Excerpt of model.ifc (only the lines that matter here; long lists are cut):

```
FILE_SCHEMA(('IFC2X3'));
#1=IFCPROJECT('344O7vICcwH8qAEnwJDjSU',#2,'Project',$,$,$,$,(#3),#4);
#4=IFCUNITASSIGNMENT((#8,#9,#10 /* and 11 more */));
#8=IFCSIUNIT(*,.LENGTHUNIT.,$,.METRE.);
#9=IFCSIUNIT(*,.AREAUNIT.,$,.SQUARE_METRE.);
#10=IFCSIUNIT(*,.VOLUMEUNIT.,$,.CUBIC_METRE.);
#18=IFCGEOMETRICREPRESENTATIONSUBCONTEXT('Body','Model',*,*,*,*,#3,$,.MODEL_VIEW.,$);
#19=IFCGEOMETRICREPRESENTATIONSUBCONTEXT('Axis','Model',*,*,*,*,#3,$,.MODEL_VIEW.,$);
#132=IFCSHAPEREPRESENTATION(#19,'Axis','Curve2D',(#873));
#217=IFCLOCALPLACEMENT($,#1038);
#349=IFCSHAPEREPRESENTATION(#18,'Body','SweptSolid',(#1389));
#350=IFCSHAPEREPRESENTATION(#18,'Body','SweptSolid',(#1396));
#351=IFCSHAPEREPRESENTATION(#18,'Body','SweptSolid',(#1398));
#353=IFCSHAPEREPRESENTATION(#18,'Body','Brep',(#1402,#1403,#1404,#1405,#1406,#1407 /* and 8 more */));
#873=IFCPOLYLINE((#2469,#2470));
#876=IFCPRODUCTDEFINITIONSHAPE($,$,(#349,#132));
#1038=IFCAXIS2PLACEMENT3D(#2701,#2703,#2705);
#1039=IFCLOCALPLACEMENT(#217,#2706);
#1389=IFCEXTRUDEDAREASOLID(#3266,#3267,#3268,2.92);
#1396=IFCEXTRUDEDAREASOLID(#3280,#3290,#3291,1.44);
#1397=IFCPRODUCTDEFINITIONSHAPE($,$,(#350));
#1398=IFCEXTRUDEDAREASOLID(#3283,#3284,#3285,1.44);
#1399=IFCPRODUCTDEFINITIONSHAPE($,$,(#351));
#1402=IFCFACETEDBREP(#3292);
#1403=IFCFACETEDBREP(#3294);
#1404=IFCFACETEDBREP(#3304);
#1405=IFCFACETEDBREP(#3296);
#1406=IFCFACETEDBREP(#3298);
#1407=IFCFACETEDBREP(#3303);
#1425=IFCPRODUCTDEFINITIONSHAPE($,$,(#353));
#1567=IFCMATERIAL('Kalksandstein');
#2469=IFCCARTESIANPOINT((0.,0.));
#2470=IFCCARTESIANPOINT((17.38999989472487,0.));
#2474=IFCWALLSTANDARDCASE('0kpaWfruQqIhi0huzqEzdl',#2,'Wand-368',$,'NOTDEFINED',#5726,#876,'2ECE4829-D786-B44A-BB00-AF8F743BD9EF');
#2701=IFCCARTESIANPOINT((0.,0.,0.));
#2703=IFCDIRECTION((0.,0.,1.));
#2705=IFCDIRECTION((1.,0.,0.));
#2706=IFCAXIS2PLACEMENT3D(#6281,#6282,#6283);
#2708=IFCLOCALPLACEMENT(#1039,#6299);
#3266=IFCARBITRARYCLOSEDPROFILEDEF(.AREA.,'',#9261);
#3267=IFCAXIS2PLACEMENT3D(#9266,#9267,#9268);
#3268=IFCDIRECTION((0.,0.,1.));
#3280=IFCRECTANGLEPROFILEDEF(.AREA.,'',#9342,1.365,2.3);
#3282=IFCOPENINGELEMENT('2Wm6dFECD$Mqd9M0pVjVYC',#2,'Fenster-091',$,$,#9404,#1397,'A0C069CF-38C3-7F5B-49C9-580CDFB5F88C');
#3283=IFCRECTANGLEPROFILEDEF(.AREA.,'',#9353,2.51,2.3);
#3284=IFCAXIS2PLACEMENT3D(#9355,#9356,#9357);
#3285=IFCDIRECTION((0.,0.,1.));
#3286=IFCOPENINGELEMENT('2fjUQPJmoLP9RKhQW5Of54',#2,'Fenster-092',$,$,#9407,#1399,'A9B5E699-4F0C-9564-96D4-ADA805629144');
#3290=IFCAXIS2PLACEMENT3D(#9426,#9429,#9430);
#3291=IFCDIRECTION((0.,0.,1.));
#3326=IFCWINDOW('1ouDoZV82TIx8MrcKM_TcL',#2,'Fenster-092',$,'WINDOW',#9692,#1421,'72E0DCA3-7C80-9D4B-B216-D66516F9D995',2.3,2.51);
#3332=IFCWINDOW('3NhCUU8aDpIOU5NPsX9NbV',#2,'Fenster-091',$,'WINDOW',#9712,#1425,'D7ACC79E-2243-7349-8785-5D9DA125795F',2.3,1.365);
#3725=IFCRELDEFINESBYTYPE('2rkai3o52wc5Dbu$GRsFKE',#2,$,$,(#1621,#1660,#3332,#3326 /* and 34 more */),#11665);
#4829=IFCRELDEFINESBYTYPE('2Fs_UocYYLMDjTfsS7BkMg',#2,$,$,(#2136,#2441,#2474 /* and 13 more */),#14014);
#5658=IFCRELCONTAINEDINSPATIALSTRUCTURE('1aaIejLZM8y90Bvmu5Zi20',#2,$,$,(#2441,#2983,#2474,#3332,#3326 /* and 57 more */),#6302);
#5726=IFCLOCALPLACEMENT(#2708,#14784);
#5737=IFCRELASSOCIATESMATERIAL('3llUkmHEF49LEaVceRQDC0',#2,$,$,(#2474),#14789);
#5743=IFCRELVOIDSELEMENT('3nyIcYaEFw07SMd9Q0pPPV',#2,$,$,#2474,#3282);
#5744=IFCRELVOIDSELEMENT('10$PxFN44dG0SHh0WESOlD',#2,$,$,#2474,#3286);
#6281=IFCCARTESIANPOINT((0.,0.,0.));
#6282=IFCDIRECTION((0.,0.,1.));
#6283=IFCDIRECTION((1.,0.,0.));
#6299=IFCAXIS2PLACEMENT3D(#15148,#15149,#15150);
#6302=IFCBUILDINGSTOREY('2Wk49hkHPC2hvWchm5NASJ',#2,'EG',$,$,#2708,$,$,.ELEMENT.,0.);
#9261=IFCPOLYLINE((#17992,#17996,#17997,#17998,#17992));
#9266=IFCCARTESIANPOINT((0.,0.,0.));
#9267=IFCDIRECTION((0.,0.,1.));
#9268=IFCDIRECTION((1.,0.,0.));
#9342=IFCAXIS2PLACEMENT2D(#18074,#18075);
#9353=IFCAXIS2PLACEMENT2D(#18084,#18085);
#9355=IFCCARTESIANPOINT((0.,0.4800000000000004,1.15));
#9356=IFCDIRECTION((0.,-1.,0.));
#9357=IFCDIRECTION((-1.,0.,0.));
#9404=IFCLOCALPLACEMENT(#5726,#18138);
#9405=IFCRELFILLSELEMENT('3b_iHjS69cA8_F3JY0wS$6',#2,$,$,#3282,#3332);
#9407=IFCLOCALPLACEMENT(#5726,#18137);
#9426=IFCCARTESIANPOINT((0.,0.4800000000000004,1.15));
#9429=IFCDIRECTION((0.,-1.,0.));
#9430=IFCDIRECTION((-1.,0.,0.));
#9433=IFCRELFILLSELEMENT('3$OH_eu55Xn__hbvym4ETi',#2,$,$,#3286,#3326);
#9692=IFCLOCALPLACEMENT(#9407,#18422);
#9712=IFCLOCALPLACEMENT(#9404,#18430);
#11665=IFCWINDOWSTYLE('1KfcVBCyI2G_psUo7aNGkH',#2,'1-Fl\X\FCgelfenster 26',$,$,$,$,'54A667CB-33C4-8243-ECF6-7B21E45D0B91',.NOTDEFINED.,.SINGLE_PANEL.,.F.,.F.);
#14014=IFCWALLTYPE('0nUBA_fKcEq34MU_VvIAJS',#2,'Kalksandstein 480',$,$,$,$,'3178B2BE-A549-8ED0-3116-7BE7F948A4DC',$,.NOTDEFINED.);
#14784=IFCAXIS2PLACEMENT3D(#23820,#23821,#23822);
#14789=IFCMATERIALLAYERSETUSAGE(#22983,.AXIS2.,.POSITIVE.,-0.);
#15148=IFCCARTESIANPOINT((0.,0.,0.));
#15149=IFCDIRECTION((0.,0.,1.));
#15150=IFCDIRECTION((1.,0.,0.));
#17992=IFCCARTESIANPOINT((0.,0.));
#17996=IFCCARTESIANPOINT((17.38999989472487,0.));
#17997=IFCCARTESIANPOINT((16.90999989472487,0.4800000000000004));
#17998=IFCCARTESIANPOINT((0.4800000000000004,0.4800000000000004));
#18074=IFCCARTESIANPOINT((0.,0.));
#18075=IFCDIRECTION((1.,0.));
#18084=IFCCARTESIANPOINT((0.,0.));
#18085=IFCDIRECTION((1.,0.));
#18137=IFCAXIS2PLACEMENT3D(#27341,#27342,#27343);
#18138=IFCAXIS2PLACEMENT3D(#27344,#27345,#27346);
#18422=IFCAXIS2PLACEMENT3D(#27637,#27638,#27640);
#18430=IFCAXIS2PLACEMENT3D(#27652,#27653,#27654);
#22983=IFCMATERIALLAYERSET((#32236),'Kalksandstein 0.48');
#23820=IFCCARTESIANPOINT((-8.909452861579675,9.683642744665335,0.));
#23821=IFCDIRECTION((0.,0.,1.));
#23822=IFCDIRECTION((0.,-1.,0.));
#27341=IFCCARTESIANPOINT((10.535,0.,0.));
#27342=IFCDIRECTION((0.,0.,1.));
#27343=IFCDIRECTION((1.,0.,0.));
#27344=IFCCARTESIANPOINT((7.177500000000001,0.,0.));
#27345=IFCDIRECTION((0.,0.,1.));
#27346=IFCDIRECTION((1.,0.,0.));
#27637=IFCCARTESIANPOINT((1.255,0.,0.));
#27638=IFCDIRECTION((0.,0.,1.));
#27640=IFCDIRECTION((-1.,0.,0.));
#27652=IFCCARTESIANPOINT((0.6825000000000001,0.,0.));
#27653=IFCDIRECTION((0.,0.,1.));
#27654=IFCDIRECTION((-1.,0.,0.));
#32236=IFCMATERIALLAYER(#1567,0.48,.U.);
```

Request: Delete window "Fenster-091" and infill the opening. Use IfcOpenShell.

```python
import ifcopenshell
import ifcopenshell.api.feature
import ifcopenshell.api.root
import ifcopenshell.geom
import ifcopenshell.util.shape

model = ifcopenshell.open("model.ifc")
settings = ifcopenshell.geom.settings()


def volume(element):
    """Net volume in cubic metres, openings subtracted."""
    shape = ifcopenshell.geom.create_shape(settings, element)
    return ifcopenshell.util.shape.get_volume(shape.geometry)


window = model.by_id(3332)
opening = window.FillsVoids[0].RelatingOpeningElement
wall = opening.VoidsElements[0].RelatingBuildingElement
before = volume(wall)

ifcopenshell.api.root.remove_product(model, product=window)
ifcopenshell.api.feature.remove_feature(model, feature=opening)

after = volume(wall)

print(f"wall volume {before:.3f} -> {after:.3f} m3")

model.write("model_updated.ifc")
```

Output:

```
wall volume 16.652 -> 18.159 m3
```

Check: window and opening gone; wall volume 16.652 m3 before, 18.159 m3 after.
